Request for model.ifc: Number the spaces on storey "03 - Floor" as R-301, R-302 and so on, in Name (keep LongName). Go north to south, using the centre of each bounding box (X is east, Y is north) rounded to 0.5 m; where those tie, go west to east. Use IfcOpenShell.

First a look at what the model holds.

```python
import ifcopenshell
import ifcopenshell.util.element
import ifcopenshell.util.placement

model = ifcopenshell.open("model.ifc")
print(model.schema)
storey = next(s for s in model.by_type("IfcBuildingStorey") if s.Name == "03 - Floor")
spaces = [e for e in ifcopenshell.util.element.get_decomposition(storey) if e.is_a("IfcSpace")]
for e in sorted(spaces, key=lambda e: e.id()):
    origin = ifcopenshell.util.placement.get_local_placement(e.ObjectPlacement)[:3, 3]
    print(e.id(), e.Name, e.LongName, origin.round(2) + 0.0, sep=" | ")
```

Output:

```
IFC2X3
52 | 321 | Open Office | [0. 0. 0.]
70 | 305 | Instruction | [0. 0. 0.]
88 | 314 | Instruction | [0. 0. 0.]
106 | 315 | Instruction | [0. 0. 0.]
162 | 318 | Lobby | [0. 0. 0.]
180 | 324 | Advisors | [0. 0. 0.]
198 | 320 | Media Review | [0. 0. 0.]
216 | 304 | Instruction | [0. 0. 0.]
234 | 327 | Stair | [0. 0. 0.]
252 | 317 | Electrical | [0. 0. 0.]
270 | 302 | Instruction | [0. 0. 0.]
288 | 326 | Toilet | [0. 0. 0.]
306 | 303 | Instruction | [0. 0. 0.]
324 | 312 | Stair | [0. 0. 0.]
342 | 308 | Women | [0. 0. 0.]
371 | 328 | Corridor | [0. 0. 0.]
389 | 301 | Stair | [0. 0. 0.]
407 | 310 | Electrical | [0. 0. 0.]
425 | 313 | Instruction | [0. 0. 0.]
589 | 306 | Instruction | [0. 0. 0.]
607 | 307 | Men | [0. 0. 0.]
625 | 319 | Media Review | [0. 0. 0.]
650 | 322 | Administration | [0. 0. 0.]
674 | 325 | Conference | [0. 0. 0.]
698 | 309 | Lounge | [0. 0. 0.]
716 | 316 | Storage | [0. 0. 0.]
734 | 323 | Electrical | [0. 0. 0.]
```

```python
import ifcopenshell
import ifcopenshell.geom
import ifcopenshell.util.element
import ifcopenshell.util.shape

model = ifcopenshell.open("model.ifc")
settings = ifcopenshell.geom.settings()
settings.set("use-world-coords", True)


def centre(element):
    shape = ifcopenshell.geom.create_shape(settings, element)
    return ifcopenshell.util.shape.get_bbox_centroid(shape.geometry)


storey = next(s for s in model.by_type("IfcBuildingStorey") if s.Name == "03 - Floor")
spaces = [e for e in ifcopenshell.util.element.get_decomposition(storey) if e.is_a("IfcSpace")]

# Insertion points can sit at a corner or the storey origin, so sort by the geometry (in metres).
centres = {e: centre(e) for e in spaces}
spaces.sort(key=lambda e: (-round(centres[e][1] / 0.5), centres[e][0]))

for i, e in enumerate(spaces, start=1):
    number = f"R-3{i:02d}"
    e.Name = number
    print(e.id(), number)

model.write("model-out.ifc")
```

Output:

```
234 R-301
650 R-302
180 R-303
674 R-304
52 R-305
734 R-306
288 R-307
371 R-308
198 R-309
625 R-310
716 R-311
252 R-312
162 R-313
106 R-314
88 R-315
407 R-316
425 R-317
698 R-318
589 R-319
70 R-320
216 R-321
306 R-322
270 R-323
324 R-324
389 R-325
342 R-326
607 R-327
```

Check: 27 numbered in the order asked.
